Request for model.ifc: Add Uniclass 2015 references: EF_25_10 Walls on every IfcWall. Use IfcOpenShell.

First a look at what the model holds.

```python
import ifcopenshell

model = ifcopenshell.open("model.ifc")
print(model.schema)
print("classifications:", [c.Name for c in model.by_type("IfcClassification")])
for ifc_class in ("IfcDoor", "IfcRoof", "IfcStair", "IfcWall", "IfcWindow"):
    print(ifc_class, len(model.by_type(ifc_class)))
```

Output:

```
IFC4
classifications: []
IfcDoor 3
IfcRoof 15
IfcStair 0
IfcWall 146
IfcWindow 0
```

```python
import ifcopenshell
import ifcopenshell.api.classification

model = ifcopenshell.open("model.ifc")

system = ifcopenshell.api.classification.add_classification(model, classification="Uniclass 2015")

codes = {
    "IfcWall": ("EF_25_10", "Walls"),
}
for ifc_class, (code, name) in codes.items():
    products = model.by_type(ifc_class)
    ifcopenshell.api.classification.add_reference(
        model, products=products, classification=system, identification=code, name=name
    )
    print(code, len(products))

model.write("model_edited.ifc")
```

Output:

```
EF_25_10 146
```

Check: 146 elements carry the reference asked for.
